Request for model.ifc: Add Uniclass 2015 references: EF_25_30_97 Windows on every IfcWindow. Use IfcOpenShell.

First a look at what the model holds.

```python
import ifcopenshell

model = ifcopenshell.open("model.ifc")
print(model.schema)
print("classifications:", [c.Name for c in model.by_type("IfcClassification")])
for ifc_class in ("IfcDoor", "IfcRoof", "IfcStair", "IfcWall", "IfcWindow"):
    print(ifc_class, len(model.by_type(ifc_class)))
```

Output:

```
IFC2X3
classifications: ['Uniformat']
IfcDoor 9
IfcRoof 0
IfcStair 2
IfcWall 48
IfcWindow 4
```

```python
import ifcopenshell
import ifcopenshell.api.classification

model = ifcopenshell.open("model.ifc")

# IFC2X3 requires Source and Edition and has no link from the project to the system.
system = model.create_entity("IfcClassification", Source="NBS", Edition="2015", Name="Uniclass 2015")

codes = {
    "IfcWindow": ("EF_25_30_97", "Windows"),
}
for ifc_class, (code, name) in codes.items():
    products = model.by_type(ifc_class)
    ifcopenshell.api.classification.add_reference(
        model, products=products, classification=system, identification=code, name=name
    )
    print(code, len(products))

model.write("model_rev.ifc")
```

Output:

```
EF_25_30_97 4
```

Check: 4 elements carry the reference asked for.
